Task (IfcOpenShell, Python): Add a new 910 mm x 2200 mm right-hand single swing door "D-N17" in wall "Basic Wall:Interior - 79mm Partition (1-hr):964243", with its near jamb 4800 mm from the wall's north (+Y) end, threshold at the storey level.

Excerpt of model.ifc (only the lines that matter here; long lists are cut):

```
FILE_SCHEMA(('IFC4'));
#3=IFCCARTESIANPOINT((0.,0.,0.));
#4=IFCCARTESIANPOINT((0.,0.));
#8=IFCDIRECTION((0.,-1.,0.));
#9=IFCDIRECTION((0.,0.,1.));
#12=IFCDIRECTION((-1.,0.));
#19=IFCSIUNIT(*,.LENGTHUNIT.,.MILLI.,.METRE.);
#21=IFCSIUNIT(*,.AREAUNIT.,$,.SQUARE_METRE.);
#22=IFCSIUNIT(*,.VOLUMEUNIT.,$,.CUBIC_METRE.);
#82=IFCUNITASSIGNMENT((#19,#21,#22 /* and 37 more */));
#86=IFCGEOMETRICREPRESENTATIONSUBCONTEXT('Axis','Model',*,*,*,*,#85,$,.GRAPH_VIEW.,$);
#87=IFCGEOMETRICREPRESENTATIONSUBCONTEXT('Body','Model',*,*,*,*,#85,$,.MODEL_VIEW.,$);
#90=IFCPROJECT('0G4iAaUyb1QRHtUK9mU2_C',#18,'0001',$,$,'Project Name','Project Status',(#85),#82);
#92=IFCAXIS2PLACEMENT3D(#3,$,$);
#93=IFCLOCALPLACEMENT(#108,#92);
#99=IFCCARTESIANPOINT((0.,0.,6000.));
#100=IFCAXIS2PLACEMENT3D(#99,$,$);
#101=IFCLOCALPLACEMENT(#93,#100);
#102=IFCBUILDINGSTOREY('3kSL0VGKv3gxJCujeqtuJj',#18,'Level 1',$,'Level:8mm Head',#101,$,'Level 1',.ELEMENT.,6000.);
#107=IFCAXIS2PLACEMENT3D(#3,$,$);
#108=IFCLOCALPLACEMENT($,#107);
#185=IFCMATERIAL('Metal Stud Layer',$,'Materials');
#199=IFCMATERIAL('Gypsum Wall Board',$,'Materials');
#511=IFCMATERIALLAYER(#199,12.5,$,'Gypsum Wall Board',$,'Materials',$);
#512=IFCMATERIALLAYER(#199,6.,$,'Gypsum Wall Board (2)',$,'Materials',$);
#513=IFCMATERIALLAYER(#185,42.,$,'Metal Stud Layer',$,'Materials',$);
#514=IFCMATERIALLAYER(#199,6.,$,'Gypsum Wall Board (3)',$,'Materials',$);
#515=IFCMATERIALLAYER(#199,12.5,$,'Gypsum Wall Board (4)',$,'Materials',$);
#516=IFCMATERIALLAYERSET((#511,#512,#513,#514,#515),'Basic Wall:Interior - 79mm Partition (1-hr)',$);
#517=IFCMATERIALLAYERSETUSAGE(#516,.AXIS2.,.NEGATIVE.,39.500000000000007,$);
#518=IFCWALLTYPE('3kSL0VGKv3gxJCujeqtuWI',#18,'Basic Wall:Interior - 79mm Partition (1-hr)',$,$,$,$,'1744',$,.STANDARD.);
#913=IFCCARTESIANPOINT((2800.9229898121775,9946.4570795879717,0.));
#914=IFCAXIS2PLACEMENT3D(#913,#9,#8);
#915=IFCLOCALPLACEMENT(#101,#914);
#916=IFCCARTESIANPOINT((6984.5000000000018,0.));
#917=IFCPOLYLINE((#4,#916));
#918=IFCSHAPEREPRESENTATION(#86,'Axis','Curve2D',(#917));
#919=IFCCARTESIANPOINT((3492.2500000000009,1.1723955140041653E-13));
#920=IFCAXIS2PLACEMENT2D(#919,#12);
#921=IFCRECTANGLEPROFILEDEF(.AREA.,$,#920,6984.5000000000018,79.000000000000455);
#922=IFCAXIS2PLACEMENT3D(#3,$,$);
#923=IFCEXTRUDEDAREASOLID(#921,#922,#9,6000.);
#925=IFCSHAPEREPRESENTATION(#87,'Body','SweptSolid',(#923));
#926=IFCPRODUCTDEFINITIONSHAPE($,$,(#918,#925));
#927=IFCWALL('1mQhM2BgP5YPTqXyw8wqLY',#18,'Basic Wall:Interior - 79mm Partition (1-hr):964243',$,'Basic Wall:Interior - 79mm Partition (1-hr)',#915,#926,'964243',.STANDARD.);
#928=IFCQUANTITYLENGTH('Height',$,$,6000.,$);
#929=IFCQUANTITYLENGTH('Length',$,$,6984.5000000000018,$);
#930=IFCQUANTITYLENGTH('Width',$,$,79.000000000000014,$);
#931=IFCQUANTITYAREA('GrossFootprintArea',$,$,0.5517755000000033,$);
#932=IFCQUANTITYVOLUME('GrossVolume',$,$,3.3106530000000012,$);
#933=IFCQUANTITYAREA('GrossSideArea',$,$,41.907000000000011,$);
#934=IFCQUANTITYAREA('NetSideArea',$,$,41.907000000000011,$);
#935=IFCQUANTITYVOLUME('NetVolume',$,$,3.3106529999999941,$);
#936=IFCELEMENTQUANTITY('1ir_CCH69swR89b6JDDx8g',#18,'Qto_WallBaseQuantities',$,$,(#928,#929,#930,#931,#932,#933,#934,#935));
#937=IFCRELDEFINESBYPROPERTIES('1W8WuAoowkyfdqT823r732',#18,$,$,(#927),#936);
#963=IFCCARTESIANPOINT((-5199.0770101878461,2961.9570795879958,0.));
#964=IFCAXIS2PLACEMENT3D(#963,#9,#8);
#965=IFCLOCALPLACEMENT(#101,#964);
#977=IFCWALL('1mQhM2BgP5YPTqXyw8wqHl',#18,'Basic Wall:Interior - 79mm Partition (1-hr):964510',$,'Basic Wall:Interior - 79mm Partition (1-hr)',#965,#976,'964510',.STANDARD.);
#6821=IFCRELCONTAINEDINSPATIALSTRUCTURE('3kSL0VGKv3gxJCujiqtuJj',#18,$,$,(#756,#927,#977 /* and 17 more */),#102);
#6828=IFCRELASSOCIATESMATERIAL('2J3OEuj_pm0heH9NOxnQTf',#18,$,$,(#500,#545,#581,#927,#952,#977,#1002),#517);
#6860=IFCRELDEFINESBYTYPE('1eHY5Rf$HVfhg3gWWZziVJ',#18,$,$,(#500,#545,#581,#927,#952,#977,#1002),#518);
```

```python
import numpy as np
import ifcopenshell
import ifcopenshell.api.feature
import ifcopenshell.api.geometry
import ifcopenshell.api.pset
import ifcopenshell.api.root
import ifcopenshell.api.spatial
import ifcopenshell.geom
import ifcopenshell.util.element
import ifcopenshell.util.placement
import ifcopenshell.util.representation
import ifcopenshell.util.shape
import ifcopenshell.util.unit

model = ifcopenshell.open("model.ifc")
unit_scale = ifcopenshell.util.unit.calculate_unit_scale(model)
area_scale = ifcopenshell.util.unit.calculate_unit_scale(model, "AREAUNIT")
volume_scale = ifcopenshell.util.unit.calculate_unit_scale(model, "VOLUMEUNIT")
settings = ifcopenshell.geom.settings()


def volume(element):
    """Net volume in cubic metres, openings subtracted."""
    shape = ifcopenshell.geom.create_shape(settings, element)
    return ifcopenshell.util.shape.get_volume(shape.geometry)


wall = model.by_guid("1mQhM2BgP5YPTqXyw8wqLY")
storey = ifcopenshell.util.element.get_container(wall, ifc_class="IfcBuildingStorey")
context = ifcopenshell.util.representation.get_context(model, "Model", "Body", "MODEL_VIEW")
before = volume(wall)

width, height, from_end, sill = 0.91, 2.2, 4.8, 0.0  # metres

# The wall runs along its own X axis, and the end named is its -X end.
wall_shape = ifcopenshell.geom.create_shape(settings, wall)
x, y, z = ifcopenshell.util.shape.get_vertices(wall_shape.geometry).T
start = x.min() + from_end
face, thickness = float(y.min()), float(y.max() - y.min())
wall_matrix = ifcopenshell.util.placement.get_local_placement(wall.ObjectPlacement)
level = ifcopenshell.util.placement.get_local_placement(storey.ObjectPlacement)[2, 3]


def in_wall(x, y):
    """Placement at x, y metres in the wall's axes, at sill height."""
    matrix = wall_matrix.copy()
    matrix[:, 3] = wall_matrix @ np.array([x / unit_scale, y / unit_scale, 0.0, 1.0])
    matrix[2, 3] = level + sill / unit_scale
    return matrix


# Opening: a box that overshoots both wall faces by 50 mm.
opening = ifcopenshell.api.root.create_entity(model, ifc_class="IfcOpeningElement", predefined_type="OPENING")
box = ifcopenshell.api.geometry.add_wall_representation(
    model, context=context, length=width, height=height, thickness=thickness + 0.1
)
ifcopenshell.api.geometry.assign_representation(model, product=opening, representation=box)
ifcopenshell.api.geometry.edit_object_placement(model, product=opening, matrix=in_wall(start, face - 0.05), is_si=False)
ifcopenshell.api.feature.add_feature(model, feature=opening, element=wall)

door = ifcopenshell.api.root.create_entity(model, ifc_class="IfcDoor", name="D-N17", predefined_type="DOOR")
door.OverallWidth, door.OverallHeight = width / unit_scale, height / unit_scale
door.OperationType = "SINGLE_SWING_RIGHT"
body = ifcopenshell.api.geometry.add_door_representation(
    model,
    context=context,
    overall_width=door.OverallWidth,
    overall_height=door.OverallHeight,
    operation_type="SINGLE_SWING_RIGHT",
    lining_properties={"LiningDepth": thickness / unit_scale, "ThresholdDepth": thickness / unit_scale},
)
ifcopenshell.api.geometry.assign_representation(model, product=door, representation=body)
ifcopenshell.api.spatial.assign_container(model, products=[door], relating_structure=storey)
ifcopenshell.api.feature.add_filling(model, opening=opening, element=door)

# The lining spans the wall, so the door starts at the wall face.
ifcopenshell.api.geometry.edit_object_placement(model, product=door, matrix=in_wall(start, face), is_si=False)

after = volume(wall)

# Update the wall's stored quantities.
qto = model.by_id(ifcopenshell.util.element.get_pset(wall, "Qto_WallBaseQuantities", should_inherit=False)["id"])
ifcopenshell.api.pset.edit_qto(model, qto=qto, properties={
    "NetSideArea": after / thickness / area_scale,
    "NetVolume": after / volume_scale,
})

print(f"wall volume {before:.3f} -> {after:.3f} m3")

model.write("model_rev.ifc")
```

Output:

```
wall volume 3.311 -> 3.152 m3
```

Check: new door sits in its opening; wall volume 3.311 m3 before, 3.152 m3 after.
